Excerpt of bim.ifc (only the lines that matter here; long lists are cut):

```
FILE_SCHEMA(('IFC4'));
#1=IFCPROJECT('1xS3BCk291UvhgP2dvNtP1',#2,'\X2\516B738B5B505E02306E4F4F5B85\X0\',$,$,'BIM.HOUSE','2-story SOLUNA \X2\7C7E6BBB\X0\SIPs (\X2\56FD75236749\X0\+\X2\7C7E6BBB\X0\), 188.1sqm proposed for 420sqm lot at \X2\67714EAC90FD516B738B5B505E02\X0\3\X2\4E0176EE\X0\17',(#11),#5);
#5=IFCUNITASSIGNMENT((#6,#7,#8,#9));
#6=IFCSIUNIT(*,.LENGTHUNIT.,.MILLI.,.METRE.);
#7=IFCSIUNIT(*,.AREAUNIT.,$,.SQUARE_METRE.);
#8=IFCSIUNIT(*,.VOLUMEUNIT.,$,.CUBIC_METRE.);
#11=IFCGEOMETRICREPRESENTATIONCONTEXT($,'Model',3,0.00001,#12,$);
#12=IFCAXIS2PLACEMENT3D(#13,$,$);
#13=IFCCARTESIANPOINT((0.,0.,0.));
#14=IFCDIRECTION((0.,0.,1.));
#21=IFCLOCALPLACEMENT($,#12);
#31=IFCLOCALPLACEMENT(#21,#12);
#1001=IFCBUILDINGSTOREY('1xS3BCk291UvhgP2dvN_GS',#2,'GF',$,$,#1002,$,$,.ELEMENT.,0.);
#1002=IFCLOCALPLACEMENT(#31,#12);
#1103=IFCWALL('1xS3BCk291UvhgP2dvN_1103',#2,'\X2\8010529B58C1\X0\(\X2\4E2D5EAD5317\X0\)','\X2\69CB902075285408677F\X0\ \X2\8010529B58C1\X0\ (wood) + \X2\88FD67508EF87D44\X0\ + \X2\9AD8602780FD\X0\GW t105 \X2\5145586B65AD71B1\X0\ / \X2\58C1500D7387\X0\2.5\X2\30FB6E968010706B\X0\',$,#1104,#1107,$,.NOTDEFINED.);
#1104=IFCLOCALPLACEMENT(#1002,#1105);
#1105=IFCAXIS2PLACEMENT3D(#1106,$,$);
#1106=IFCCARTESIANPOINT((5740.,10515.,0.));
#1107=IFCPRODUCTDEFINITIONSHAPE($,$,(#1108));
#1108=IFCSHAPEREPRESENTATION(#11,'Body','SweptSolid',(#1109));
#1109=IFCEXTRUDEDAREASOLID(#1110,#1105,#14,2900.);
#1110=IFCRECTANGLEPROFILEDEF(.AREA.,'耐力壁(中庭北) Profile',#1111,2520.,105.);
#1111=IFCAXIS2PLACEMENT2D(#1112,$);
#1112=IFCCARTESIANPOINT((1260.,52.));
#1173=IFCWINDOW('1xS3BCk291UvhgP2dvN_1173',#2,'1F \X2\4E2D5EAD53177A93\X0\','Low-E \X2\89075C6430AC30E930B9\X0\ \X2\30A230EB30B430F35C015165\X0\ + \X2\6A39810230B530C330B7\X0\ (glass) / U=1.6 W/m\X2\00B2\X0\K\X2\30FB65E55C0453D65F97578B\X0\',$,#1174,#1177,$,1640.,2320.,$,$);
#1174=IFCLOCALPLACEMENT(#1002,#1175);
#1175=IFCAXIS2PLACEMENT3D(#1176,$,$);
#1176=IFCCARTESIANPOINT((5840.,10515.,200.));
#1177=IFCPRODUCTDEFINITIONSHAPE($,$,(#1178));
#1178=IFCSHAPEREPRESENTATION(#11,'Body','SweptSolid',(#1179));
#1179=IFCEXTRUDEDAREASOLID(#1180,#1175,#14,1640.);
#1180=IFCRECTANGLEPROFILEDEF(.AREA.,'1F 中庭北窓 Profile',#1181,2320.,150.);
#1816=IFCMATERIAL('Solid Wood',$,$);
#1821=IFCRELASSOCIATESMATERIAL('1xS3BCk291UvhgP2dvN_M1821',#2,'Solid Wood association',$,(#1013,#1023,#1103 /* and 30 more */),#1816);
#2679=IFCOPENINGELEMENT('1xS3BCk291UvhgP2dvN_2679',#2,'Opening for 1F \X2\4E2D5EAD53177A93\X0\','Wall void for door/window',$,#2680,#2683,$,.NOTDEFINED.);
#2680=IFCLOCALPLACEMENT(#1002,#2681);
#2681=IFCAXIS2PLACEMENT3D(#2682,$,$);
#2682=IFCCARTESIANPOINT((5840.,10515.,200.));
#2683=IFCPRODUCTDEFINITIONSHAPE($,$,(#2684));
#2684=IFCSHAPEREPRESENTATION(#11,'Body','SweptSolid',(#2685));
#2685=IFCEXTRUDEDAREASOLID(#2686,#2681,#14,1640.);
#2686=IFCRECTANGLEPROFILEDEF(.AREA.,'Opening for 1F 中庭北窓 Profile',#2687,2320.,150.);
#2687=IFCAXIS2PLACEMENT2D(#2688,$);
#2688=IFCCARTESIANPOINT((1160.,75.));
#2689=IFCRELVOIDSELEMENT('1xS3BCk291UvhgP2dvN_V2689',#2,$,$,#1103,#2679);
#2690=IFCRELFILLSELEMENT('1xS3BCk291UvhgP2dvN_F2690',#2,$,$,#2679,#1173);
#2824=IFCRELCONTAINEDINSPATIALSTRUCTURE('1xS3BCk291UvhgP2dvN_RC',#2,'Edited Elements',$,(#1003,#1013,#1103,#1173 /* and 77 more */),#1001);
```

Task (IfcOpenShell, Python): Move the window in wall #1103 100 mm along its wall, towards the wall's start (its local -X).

```python
import ifcopenshell
import ifcopenshell.api.geometry
import ifcopenshell.util.placement
import ifcopenshell.util.unit

model = ifcopenshell.open("bim.ifc")
unit_scale = ifcopenshell.util.unit.calculate_unit_scale(model)

window = model.by_id(1173)
opening = window.FillsVoids[0].RelatingOpeningElement
wall = opening.VoidsElements[0].RelatingBuildingElement

wall_matrix = ifcopenshell.util.placement.get_local_placement(wall.ObjectPlacement)
shift = wall_matrix[:3, 0] * -0.1 / unit_scale
before = ifcopenshell.util.placement.get_local_placement(window.ObjectPlacement)[:3, 3].copy()

# The window is not placed relative to its opening, so move both.
for product in (opening, window):
    matrix = ifcopenshell.util.placement.get_local_placement(product.ObjectPlacement)
    matrix[:3, 3] += shift
    ifcopenshell.api.geometry.edit_object_placement(model, product=product, matrix=matrix, is_si=False)

after = ifcopenshell.util.placement.get_local_placement(window.ObjectPlacement)[:3, 3]
print("window moved by", (after - before).round(3) + 0.0)

model.write("bim-out.ifc")
```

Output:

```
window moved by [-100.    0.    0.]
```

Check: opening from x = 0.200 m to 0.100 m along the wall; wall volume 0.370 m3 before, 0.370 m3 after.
